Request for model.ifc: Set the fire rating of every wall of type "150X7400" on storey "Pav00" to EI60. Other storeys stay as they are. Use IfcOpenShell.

First a look at what the model holds.

```python
import ifcopenshell
import ifcopenshell.util.element

model = ifcopenshell.open("model.ifc")
print(model.schema)
storey = next(s for s in model.by_type("IfcBuildingStorey") if s.Name == "Pav00")
walls = [e for e in ifcopenshell.util.element.get_decomposition(storey) if e.is_a("IfcWall")]
seen = {}
for e in walls:
    element_type = ifcopenshell.util.element.get_type(e)
    key = (element_type.Name if element_type != e and element_type else None, ifcopenshell.util.element.get_pset(e, "Pset_WallCommon", "FireRating"))
    seen[key] = seen.get(key, 0) + 1
for (name, value), count in sorted(seen.items(), key=str):
    print(count, "x", name, "|", value)
```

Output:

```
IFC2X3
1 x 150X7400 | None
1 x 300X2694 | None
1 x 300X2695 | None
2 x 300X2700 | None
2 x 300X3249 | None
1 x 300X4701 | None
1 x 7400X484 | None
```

```python
import ifcopenshell
import ifcopenshell.api.pset
import ifcopenshell.util.element

model = ifcopenshell.open("model.ifc")

storey = next(s for s in model.by_type("IfcBuildingStorey") if s.Name == "Pav00")
walls = [e for e in ifcopenshell.util.element.get_decomposition(storey) if e.is_a("IfcWall")]

count = 0
for e in walls:
    element_type = ifcopenshell.util.element.get_type(e)
    if element_type in (None, e) or element_type.Name != "150X7400":
        continue
    # add_pset returns the element's existing set when there is one.
    pset = ifcopenshell.api.pset.add_pset(model, product=e, name="Pset_WallCommon")
    ifcopenshell.api.pset.edit_pset(model, pset=pset, properties={"FireRating": "EI60"})
    count += 1

print(count, "walls updated")

model.write("model_rev.ifc")
```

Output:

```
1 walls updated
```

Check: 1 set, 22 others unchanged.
